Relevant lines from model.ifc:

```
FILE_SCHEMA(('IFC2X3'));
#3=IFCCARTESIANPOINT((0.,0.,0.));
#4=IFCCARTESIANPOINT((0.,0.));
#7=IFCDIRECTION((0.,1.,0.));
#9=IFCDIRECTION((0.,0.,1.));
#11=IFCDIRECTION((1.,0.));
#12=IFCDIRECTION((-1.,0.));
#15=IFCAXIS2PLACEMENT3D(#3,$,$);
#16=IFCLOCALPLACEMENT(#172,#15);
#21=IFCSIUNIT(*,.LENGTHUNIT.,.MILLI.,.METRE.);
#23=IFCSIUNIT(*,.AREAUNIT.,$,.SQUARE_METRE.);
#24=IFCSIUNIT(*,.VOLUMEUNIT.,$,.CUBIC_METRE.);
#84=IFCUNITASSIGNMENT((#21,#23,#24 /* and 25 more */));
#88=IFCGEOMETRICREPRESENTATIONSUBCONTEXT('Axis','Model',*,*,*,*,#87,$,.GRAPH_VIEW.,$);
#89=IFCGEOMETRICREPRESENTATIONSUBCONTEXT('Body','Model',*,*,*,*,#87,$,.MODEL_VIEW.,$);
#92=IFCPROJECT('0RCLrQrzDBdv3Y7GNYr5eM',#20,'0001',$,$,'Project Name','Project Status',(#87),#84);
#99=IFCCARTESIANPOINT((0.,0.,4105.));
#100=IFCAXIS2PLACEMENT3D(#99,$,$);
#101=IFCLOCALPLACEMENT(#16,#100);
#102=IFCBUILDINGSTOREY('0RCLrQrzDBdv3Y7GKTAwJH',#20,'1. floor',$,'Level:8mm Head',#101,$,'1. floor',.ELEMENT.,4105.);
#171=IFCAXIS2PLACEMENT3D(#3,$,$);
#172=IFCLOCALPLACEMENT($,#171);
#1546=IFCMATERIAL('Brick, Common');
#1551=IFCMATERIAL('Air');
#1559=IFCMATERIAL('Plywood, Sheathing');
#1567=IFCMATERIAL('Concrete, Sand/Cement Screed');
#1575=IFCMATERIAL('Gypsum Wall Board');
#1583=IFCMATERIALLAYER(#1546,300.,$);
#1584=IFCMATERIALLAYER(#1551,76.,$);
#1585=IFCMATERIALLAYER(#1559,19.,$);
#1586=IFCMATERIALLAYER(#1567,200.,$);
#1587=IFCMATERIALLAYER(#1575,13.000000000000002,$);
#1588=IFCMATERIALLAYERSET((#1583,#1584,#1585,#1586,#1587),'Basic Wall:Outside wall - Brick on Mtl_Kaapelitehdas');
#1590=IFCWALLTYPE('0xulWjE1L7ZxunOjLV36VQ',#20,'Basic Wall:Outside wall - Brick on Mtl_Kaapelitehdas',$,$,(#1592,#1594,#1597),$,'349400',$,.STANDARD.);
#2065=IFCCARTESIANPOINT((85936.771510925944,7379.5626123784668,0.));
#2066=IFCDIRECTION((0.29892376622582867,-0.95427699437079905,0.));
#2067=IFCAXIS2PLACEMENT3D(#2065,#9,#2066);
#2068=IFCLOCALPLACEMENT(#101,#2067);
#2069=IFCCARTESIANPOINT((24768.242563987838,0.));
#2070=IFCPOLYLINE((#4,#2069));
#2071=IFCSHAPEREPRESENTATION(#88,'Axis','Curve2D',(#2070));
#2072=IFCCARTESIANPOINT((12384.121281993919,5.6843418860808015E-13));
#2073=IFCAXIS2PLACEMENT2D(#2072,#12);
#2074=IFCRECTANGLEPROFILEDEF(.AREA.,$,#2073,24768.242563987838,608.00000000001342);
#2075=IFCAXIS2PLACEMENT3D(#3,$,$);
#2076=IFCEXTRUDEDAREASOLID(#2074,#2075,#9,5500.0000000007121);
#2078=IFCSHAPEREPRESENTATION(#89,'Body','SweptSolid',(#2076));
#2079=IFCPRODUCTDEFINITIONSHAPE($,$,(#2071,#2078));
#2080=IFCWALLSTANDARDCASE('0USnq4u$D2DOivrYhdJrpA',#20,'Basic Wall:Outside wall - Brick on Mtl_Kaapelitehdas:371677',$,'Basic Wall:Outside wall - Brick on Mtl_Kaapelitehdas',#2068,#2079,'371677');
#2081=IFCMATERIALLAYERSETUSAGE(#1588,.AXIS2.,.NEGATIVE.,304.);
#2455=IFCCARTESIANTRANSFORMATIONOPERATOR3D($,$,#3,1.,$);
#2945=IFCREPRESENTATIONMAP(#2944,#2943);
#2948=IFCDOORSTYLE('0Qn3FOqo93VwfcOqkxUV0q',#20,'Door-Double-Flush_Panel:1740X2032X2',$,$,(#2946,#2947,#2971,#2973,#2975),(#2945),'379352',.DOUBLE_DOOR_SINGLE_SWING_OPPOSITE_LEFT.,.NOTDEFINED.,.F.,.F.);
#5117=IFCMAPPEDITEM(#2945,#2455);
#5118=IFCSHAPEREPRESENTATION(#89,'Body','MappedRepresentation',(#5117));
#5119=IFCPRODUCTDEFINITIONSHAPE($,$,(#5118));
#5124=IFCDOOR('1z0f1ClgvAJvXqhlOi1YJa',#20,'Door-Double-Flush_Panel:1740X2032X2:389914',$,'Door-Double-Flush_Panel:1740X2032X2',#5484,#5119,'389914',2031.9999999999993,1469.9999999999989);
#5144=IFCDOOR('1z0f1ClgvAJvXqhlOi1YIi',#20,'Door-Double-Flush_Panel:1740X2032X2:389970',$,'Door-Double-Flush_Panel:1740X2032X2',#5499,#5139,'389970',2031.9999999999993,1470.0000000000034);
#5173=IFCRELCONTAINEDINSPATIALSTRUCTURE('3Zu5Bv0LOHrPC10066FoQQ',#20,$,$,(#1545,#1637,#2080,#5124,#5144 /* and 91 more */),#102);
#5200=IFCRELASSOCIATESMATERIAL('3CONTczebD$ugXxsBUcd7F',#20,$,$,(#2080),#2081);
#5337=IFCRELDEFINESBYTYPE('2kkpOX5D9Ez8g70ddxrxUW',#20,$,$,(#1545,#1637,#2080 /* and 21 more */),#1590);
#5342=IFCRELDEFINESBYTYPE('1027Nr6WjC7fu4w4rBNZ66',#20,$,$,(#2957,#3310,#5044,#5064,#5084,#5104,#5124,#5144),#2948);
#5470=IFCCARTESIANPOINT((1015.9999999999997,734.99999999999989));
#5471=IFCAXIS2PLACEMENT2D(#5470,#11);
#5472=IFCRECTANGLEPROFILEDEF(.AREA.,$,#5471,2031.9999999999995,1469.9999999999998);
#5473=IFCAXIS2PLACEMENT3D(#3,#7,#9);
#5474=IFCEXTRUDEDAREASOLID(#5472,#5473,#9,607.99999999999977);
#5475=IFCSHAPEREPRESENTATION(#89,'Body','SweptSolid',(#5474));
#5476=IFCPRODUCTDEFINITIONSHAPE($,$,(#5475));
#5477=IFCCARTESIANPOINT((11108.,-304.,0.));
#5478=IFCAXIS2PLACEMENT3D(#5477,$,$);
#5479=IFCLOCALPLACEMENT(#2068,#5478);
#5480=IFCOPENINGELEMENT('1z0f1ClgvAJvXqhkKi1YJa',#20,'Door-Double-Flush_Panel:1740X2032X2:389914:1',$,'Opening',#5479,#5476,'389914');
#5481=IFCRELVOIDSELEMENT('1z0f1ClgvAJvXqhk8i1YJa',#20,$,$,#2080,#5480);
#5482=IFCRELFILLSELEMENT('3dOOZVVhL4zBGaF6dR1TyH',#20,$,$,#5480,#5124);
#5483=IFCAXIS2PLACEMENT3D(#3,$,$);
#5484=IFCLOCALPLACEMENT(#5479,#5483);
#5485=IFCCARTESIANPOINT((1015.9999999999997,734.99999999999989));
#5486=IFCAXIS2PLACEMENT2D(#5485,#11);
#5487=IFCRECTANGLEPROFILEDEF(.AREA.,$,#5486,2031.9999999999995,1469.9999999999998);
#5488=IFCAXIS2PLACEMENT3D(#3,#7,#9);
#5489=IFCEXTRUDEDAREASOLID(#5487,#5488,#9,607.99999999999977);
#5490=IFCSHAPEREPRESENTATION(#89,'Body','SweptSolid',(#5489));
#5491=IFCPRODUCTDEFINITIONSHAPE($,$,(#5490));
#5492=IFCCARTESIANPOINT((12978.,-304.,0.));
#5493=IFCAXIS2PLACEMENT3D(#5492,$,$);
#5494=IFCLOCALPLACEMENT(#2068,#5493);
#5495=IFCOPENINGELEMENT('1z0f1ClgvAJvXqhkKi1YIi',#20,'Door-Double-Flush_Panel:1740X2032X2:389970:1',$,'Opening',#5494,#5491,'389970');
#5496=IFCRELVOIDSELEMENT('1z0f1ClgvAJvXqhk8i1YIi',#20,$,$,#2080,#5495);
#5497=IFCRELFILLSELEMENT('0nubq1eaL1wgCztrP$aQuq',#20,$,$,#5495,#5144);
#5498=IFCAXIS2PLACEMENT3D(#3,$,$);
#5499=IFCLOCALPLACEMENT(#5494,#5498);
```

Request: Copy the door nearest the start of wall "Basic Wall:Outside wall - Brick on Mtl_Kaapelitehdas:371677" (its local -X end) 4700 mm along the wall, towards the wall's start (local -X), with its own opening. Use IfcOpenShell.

```python
import ifcopenshell
import ifcopenshell.api.feature
import ifcopenshell.api.geometry
import ifcopenshell.api.root
import ifcopenshell.geom
import ifcopenshell.util.element
import ifcopenshell.util.placement
import ifcopenshell.util.shape
import ifcopenshell.util.unit

model = ifcopenshell.open("model.ifc")
unit_scale = ifcopenshell.util.unit.calculate_unit_scale(model)
settings = ifcopenshell.geom.settings()


def volume(element):
    """Net volume in cubic metres, openings subtracted."""
    shape = ifcopenshell.geom.create_shape(settings, element)
    return ifcopenshell.util.shape.get_volume(shape.geometry)


def reuse_history(source, copy):
    """copy_class also copies each property set's owner history, people and application; keep the originals."""
    for rel in copy.IsDefinedBy:
        if rel.is_a("IfcRelDefinesByProperties") and (history := rel.RelatingPropertyDefinition.OwnerHistory):
            rel.RelatingPropertyDefinition.OwnerHistory = source.OwnerHistory
            ifcopenshell.util.element.remove_deep2(model, history)


door = model.by_guid("1z0f1ClgvAJvXqhlOi1YJa")
opening = door.FillsVoids[0].RelatingOpeningElement
wall = opening.VoidsElements[0].RelatingBuildingElement
before = volume(wall)
shift = ifcopenshell.util.placement.get_local_placement(wall.ObjectPlacement)[:3, 0] * -4.7 / unit_scale

# copy_class copies the void relationship, type, container and properties, but no geometry.
new_opening = ifcopenshell.api.root.copy_class(model, product=opening)
new_opening.Representation = ifcopenshell.util.element.copy_deep(
    model, opening.Representation, exclude=["IfcGeometricRepresentationContext", "IfcRepresentationMap"]
)
new_opening.Name = "Door-Double-Flush_Panel:1740X2032X2"
new_opening.Tag = None
new_door = ifcopenshell.api.root.copy_class(model, product=door)
new_door.Representation = ifcopenshell.util.element.copy_deep(
    model, door.Representation, exclude=["IfcGeometricRepresentationContext", "IfcRepresentationMap"]
)
new_door.Name = "Door-Double-Flush_Panel:1740X2032X2"
new_door.Tag = None
reuse_history(door, new_door)
fills = ifcopenshell.api.feature.add_filling(model, opening=new_opening, element=new_door)
fills.OwnerHistory = new_door.OwnerHistory  # required in IFC2X3

for old, new in ((opening, new_opening), (door, new_door)):
    matrix = ifcopenshell.util.placement.get_local_placement(old.ObjectPlacement)
    matrix[:3, 3] += shift
    ifcopenshell.api.geometry.edit_object_placement(model, product=new, matrix=matrix, is_si=False)

after = volume(wall)

print(f"wall volume {before:.3f} -> {after:.3f} m3")

model.write("model-out.ifc")
```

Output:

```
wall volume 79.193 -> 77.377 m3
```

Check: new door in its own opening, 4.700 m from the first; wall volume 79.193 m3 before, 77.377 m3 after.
